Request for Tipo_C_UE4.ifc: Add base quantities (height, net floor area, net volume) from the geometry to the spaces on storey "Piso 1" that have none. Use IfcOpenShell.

First a look at what the model holds.

```python
import ifcopenshell
import ifcopenshell.util.element
import ifcopenshell.util.unit

model = ifcopenshell.open("Tipo_C_UE4.ifc")
print(model.schema)
for unit_type in ("LENGTHUNIT", "AREAUNIT", "VOLUMEUNIT"):
    print(unit_type, ifcopenshell.util.unit.calculate_unit_scale(model, unit_type))
storey = next(s for s in model.by_type("IfcBuildingStorey") if s.Name == "Piso 1")
spaces = [e for e in ifcopenshell.util.element.get_decomposition(storey) if e.is_a("IfcSpace")]
for e in sorted(spaces, key=lambda e: e.id()):
    print(e.id(), e.is_a(), e.Name, list(ifcopenshell.util.element.get_psets(e, qtos_only=True)), sep=" | ")
```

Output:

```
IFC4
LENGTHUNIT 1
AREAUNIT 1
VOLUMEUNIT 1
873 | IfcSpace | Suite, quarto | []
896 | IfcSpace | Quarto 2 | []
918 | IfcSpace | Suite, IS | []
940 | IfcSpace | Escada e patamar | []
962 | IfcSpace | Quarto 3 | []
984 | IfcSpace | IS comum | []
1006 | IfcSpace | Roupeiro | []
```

```python
import ifcopenshell
import ifcopenshell.api.pset
import ifcopenshell.geom
import ifcopenshell.util.element
import ifcopenshell.util.shape
import ifcopenshell.util.unit

model = ifcopenshell.open("Tipo_C_UE4.ifc")
unit_scale = ifcopenshell.util.unit.calculate_unit_scale(model)
area_scale = ifcopenshell.util.unit.calculate_unit_scale(model, "AREAUNIT")
volume_scale = ifcopenshell.util.unit.calculate_unit_scale(model, "VOLUMEUNIT")
settings = ifcopenshell.geom.settings()

storey = next(s for s in model.by_type("IfcBuildingStorey") if s.Name == "Piso 1")
spaces = [e for e in ifcopenshell.util.element.get_decomposition(storey) if e.is_a("IfcSpace")]

for e in sorted(spaces, key=lambda e: e.id()):
    if ifcopenshell.util.element.get_psets(e, qtos_only=True, should_inherit=False):
        continue
    # Geometry comes back in metres, in the element's own axes.
    shape = ifcopenshell.geom.create_shape(settings, e)
    values = {
        "Height": ifcopenshell.util.shape.get_z(shape.geometry) / unit_scale,
        "NetFloorArea": ifcopenshell.util.shape.get_footprint_area(shape.geometry) / area_scale,
        "NetVolume": ifcopenshell.util.shape.get_volume(shape.geometry) / volume_scale,
    }
    qto = ifcopenshell.api.pset.add_qto(model, product=e, name="Qto_SpaceBaseQuantities")
    ifcopenshell.api.pset.edit_qto(model, qto=qto, properties=values)
    print(e.id(), {k: round(v, 3) for k, v in values.items()})

model.write("Tipo_C_UE4_v2.ifc")
```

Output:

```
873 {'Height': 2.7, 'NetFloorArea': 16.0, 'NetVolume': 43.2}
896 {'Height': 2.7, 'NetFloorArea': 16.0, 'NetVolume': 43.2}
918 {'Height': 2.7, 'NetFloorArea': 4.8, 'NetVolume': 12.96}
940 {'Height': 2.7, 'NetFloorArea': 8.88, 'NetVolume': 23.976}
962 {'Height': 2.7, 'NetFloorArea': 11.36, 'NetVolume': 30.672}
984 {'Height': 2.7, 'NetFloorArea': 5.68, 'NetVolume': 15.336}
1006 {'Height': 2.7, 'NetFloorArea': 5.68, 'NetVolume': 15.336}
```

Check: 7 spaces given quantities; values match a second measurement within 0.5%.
